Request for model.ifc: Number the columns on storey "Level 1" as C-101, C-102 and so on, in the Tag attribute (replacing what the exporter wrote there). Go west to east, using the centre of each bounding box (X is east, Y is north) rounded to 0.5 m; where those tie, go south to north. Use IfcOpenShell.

First a look at what the model holds.

```python
import ifcopenshell
import ifcopenshell.util.element
import ifcopenshell.util.placement

model = ifcopenshell.open("model.ifc")
print(model.schema)
storey = next(s for s in model.by_type("IfcBuildingStorey") if s.Name == "Level 1")
columns = [e for e in ifcopenshell.util.element.get_decomposition(storey) if e.is_a("IfcColumn")]
for e in sorted(columns, key=lambda e: e.id()):
    origin = ifcopenshell.util.placement.get_local_placement(e.ObjectPlacement)[:3, 3]
    print(e.id(), e.Tag, e.Name, origin.round(2) + 0.0, sep=" | ")
```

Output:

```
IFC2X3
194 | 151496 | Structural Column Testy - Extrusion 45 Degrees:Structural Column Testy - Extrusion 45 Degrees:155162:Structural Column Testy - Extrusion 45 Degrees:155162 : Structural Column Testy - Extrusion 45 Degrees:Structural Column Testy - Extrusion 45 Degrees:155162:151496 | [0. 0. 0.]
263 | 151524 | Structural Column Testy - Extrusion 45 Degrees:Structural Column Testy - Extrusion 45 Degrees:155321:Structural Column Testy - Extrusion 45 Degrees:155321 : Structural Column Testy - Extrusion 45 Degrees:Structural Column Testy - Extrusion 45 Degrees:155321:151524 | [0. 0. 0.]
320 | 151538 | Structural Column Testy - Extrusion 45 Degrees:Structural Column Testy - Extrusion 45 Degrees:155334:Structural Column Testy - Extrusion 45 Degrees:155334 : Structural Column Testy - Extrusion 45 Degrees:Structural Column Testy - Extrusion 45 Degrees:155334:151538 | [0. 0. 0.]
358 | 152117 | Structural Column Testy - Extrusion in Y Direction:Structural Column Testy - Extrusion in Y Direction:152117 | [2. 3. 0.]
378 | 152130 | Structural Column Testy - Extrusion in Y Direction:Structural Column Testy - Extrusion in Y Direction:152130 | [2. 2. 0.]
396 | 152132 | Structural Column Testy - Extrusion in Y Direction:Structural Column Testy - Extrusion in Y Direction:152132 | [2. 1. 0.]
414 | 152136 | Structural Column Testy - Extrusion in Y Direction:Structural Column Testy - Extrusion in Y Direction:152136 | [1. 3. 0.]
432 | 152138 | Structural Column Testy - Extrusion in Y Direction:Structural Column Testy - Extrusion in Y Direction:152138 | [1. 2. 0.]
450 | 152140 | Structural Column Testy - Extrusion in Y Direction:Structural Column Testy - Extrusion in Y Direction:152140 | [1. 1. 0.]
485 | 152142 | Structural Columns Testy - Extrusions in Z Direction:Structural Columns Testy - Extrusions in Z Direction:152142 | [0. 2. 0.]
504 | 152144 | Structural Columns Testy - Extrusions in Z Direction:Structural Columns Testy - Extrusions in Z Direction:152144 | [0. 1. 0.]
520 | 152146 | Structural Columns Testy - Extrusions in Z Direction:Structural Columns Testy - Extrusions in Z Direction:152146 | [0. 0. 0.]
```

```python
import ifcopenshell
import ifcopenshell.geom
import ifcopenshell.util.element
import ifcopenshell.util.shape

model = ifcopenshell.open("model.ifc")
settings = ifcopenshell.geom.settings()
settings.set("use-world-coords", True)


def centre(element):
    shape = ifcopenshell.geom.create_shape(settings, element)
    return ifcopenshell.util.shape.get_bbox_centroid(shape.geometry)


storey = next(s for s in model.by_type("IfcBuildingStorey") if s.Name == "Level 1")
columns = [e for e in ifcopenshell.util.element.get_decomposition(storey) if e.is_a("IfcColumn")]

# Insertion points can sit at a corner or the storey origin, so sort by the geometry (in metres).
centres = {e: centre(e) for e in columns}
columns.sort(key=lambda e: (round(centres[e][0] / 0.5), centres[e][1]))

for i, e in enumerate(columns, start=1):
    number = f"C-1{i:02d}"
    e.Tag = number
    print(e.id(), number)

model.write("model-out.ifc")
```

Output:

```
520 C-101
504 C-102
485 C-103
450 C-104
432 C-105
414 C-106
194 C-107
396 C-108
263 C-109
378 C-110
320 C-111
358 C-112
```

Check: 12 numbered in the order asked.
